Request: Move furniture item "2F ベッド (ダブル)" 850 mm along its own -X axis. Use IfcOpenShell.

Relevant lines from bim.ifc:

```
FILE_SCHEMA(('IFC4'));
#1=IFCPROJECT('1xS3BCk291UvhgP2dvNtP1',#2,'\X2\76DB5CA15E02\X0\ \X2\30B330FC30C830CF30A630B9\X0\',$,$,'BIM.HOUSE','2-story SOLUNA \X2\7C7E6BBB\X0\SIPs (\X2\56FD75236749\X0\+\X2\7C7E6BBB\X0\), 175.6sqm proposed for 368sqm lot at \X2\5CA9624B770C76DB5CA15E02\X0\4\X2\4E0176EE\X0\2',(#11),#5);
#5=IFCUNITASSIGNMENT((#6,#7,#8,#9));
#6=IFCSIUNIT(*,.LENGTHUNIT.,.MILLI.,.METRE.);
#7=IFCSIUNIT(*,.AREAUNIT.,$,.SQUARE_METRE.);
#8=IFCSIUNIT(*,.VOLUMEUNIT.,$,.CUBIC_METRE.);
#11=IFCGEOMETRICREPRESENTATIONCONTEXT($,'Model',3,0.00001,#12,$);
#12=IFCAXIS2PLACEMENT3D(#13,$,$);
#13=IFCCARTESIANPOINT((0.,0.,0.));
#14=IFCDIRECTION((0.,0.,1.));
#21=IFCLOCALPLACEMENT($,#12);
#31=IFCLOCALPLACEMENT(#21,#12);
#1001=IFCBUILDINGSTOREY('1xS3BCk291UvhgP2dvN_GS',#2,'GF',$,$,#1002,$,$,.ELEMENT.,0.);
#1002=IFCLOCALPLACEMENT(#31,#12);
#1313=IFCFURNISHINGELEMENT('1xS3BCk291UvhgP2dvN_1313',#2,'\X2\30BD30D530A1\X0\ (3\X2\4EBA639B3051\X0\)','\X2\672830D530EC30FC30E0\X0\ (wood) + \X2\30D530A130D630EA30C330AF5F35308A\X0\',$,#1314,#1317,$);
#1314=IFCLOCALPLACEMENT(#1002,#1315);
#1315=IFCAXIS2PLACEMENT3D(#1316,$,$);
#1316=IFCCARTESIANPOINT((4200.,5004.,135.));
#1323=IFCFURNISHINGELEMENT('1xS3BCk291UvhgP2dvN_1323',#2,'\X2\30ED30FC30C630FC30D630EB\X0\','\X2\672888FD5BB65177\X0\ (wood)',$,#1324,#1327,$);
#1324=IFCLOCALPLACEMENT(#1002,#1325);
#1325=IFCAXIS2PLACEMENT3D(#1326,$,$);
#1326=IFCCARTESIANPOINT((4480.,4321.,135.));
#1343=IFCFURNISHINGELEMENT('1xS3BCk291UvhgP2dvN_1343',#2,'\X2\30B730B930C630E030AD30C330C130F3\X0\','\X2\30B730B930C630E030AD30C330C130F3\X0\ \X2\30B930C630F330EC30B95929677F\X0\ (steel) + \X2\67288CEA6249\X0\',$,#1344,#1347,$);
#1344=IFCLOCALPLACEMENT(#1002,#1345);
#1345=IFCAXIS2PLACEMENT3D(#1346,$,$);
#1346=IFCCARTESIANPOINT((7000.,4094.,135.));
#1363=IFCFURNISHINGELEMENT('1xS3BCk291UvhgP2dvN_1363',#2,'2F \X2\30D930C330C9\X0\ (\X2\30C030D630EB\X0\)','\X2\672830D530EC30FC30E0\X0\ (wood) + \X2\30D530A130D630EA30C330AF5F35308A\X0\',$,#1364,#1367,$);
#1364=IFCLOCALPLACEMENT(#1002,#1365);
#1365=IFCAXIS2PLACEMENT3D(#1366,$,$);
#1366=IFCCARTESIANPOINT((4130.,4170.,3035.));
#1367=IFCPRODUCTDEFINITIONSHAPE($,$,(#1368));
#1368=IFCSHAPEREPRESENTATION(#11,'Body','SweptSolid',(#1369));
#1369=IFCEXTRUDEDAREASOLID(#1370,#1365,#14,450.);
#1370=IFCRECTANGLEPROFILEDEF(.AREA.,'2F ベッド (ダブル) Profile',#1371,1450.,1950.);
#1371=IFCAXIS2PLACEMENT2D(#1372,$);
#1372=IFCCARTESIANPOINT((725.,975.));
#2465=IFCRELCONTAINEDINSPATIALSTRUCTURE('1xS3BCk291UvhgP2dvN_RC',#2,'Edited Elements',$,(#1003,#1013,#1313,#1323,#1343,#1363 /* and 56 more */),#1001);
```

```python
import ifcopenshell
import ifcopenshell.api.geometry
import ifcopenshell.util.placement

model = ifcopenshell.open("bim.ifc")

item = model.by_guid("1xS3BCk291UvhgP2dvN_1363")
matrix = ifcopenshell.util.placement.get_local_placement(item.ObjectPlacement)
matrix[:3, 3] -= matrix[:3, 0] * 850.0
ifcopenshell.api.geometry.edit_object_placement(model, product=item, matrix=matrix, is_si=False)

print(ifcopenshell.util.placement.get_local_placement(item.ObjectPlacement).round(3) + 0.0)

model.write("bim_updated.ifc")
```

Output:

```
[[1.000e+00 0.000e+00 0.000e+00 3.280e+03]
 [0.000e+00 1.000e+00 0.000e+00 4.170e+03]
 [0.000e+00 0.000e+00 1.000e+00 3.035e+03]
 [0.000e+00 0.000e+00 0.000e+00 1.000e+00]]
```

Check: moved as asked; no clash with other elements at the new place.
